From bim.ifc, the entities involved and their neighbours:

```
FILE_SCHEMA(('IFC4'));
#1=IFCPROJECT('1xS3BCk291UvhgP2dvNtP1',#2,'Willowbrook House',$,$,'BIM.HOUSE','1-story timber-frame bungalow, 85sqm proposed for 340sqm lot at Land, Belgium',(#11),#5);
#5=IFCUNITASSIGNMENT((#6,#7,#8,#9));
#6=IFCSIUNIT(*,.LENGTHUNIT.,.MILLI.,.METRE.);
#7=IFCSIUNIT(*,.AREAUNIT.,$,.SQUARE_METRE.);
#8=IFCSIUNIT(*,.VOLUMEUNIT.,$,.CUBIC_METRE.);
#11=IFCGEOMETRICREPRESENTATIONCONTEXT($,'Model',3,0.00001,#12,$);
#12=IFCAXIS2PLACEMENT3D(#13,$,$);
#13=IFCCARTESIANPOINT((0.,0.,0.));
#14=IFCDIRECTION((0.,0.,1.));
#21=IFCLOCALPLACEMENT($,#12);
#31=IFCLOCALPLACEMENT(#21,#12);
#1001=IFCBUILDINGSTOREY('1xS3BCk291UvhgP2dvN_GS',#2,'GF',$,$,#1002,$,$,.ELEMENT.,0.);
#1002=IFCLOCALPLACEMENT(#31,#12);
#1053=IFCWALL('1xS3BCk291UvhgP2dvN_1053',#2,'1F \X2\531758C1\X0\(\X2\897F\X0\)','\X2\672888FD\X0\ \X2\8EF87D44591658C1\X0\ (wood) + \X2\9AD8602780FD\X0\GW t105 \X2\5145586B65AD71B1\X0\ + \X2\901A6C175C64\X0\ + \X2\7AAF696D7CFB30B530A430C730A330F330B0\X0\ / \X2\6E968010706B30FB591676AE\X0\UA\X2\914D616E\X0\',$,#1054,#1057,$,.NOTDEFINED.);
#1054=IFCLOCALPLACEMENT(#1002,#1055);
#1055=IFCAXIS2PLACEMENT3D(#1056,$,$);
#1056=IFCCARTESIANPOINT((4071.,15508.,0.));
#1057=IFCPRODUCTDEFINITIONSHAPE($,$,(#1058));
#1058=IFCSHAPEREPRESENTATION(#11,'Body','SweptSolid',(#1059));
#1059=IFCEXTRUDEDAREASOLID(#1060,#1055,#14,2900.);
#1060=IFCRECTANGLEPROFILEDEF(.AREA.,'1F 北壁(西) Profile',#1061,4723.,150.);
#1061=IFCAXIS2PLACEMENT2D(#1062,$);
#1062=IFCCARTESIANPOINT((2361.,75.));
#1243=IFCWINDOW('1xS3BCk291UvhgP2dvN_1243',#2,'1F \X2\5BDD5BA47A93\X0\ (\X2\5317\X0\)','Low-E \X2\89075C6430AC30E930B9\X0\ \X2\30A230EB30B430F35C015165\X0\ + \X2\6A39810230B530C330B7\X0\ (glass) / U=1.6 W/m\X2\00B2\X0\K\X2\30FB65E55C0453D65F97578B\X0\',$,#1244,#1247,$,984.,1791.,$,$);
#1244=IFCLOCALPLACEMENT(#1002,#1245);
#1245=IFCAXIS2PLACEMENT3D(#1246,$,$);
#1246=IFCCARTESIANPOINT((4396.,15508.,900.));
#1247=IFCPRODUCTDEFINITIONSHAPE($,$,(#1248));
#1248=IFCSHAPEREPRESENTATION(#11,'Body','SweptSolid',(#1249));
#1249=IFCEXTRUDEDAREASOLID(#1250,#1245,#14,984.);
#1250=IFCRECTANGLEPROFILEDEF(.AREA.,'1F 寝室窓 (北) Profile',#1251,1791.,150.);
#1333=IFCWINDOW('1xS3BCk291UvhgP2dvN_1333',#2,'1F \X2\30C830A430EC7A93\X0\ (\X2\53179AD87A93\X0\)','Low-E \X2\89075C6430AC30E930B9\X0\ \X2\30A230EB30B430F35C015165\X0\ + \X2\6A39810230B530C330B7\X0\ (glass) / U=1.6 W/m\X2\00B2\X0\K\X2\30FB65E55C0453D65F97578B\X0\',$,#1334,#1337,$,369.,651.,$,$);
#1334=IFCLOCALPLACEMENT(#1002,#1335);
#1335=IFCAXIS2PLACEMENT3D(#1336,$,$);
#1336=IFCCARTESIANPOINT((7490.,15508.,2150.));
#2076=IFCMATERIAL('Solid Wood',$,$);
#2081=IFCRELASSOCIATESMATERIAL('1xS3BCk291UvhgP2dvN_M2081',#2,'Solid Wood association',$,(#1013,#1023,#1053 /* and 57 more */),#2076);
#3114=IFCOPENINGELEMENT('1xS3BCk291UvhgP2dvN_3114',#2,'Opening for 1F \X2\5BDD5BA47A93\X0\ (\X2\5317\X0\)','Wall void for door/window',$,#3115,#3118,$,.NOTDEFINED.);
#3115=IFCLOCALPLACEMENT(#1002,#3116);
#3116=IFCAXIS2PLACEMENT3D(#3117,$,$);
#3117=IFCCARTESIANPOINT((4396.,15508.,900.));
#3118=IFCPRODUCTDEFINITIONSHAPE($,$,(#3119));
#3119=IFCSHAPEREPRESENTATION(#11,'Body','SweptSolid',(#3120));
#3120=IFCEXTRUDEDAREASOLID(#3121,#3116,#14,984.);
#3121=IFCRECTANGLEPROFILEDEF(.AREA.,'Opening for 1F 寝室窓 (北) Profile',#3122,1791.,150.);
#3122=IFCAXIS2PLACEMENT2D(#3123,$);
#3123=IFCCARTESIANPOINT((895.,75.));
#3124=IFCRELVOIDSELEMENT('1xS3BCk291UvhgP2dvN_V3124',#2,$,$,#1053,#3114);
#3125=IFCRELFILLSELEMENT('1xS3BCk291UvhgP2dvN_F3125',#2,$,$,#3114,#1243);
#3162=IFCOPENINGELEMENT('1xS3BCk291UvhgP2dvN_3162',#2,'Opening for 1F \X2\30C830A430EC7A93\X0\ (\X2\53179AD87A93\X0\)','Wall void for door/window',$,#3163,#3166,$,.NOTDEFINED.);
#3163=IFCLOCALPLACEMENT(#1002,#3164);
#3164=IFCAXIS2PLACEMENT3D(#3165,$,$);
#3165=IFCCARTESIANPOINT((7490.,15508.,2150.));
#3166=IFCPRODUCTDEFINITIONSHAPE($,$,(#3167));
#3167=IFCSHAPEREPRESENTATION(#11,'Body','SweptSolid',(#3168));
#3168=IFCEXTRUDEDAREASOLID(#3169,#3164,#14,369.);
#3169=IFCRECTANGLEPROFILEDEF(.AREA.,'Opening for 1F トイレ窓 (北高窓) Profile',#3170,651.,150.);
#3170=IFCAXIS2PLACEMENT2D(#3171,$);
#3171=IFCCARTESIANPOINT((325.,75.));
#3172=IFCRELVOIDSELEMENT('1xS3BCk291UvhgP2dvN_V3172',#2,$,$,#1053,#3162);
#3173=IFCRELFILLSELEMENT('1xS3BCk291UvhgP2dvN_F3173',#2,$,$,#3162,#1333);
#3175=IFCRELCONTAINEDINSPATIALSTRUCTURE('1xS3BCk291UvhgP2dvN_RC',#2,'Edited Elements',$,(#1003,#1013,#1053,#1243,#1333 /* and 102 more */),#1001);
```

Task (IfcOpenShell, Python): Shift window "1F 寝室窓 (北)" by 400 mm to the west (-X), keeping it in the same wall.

```python
import ifcopenshell
import ifcopenshell.api.geometry
import ifcopenshell.util.placement

model = ifcopenshell.open("bim.ifc")

window = model.by_id(1243)
opening = window.FillsVoids[0].RelatingOpeningElement
wall = opening.VoidsElements[0].RelatingBuildingElement

wall_matrix = ifcopenshell.util.placement.get_local_placement(wall.ObjectPlacement)
shift = wall_matrix[:3, 0] * -400.0
before = ifcopenshell.util.placement.get_local_placement(window.ObjectPlacement)[:3, 3].copy()

# The window is not placed relative to its opening, so move both.
for product in (opening, window):
    matrix = ifcopenshell.util.placement.get_local_placement(product.ObjectPlacement)
    matrix[:3, 3] += shift
    ifcopenshell.api.geometry.edit_object_placement(model, product=product, matrix=matrix, is_si=False)

after = ifcopenshell.util.placement.get_local_placement(window.ObjectPlacement)[:3, 3]
print("window moved by", (after - before).round(3) + 0.0)

model.write("bim_updated.ifc")
```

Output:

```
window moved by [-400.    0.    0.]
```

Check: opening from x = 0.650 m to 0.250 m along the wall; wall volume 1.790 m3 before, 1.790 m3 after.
